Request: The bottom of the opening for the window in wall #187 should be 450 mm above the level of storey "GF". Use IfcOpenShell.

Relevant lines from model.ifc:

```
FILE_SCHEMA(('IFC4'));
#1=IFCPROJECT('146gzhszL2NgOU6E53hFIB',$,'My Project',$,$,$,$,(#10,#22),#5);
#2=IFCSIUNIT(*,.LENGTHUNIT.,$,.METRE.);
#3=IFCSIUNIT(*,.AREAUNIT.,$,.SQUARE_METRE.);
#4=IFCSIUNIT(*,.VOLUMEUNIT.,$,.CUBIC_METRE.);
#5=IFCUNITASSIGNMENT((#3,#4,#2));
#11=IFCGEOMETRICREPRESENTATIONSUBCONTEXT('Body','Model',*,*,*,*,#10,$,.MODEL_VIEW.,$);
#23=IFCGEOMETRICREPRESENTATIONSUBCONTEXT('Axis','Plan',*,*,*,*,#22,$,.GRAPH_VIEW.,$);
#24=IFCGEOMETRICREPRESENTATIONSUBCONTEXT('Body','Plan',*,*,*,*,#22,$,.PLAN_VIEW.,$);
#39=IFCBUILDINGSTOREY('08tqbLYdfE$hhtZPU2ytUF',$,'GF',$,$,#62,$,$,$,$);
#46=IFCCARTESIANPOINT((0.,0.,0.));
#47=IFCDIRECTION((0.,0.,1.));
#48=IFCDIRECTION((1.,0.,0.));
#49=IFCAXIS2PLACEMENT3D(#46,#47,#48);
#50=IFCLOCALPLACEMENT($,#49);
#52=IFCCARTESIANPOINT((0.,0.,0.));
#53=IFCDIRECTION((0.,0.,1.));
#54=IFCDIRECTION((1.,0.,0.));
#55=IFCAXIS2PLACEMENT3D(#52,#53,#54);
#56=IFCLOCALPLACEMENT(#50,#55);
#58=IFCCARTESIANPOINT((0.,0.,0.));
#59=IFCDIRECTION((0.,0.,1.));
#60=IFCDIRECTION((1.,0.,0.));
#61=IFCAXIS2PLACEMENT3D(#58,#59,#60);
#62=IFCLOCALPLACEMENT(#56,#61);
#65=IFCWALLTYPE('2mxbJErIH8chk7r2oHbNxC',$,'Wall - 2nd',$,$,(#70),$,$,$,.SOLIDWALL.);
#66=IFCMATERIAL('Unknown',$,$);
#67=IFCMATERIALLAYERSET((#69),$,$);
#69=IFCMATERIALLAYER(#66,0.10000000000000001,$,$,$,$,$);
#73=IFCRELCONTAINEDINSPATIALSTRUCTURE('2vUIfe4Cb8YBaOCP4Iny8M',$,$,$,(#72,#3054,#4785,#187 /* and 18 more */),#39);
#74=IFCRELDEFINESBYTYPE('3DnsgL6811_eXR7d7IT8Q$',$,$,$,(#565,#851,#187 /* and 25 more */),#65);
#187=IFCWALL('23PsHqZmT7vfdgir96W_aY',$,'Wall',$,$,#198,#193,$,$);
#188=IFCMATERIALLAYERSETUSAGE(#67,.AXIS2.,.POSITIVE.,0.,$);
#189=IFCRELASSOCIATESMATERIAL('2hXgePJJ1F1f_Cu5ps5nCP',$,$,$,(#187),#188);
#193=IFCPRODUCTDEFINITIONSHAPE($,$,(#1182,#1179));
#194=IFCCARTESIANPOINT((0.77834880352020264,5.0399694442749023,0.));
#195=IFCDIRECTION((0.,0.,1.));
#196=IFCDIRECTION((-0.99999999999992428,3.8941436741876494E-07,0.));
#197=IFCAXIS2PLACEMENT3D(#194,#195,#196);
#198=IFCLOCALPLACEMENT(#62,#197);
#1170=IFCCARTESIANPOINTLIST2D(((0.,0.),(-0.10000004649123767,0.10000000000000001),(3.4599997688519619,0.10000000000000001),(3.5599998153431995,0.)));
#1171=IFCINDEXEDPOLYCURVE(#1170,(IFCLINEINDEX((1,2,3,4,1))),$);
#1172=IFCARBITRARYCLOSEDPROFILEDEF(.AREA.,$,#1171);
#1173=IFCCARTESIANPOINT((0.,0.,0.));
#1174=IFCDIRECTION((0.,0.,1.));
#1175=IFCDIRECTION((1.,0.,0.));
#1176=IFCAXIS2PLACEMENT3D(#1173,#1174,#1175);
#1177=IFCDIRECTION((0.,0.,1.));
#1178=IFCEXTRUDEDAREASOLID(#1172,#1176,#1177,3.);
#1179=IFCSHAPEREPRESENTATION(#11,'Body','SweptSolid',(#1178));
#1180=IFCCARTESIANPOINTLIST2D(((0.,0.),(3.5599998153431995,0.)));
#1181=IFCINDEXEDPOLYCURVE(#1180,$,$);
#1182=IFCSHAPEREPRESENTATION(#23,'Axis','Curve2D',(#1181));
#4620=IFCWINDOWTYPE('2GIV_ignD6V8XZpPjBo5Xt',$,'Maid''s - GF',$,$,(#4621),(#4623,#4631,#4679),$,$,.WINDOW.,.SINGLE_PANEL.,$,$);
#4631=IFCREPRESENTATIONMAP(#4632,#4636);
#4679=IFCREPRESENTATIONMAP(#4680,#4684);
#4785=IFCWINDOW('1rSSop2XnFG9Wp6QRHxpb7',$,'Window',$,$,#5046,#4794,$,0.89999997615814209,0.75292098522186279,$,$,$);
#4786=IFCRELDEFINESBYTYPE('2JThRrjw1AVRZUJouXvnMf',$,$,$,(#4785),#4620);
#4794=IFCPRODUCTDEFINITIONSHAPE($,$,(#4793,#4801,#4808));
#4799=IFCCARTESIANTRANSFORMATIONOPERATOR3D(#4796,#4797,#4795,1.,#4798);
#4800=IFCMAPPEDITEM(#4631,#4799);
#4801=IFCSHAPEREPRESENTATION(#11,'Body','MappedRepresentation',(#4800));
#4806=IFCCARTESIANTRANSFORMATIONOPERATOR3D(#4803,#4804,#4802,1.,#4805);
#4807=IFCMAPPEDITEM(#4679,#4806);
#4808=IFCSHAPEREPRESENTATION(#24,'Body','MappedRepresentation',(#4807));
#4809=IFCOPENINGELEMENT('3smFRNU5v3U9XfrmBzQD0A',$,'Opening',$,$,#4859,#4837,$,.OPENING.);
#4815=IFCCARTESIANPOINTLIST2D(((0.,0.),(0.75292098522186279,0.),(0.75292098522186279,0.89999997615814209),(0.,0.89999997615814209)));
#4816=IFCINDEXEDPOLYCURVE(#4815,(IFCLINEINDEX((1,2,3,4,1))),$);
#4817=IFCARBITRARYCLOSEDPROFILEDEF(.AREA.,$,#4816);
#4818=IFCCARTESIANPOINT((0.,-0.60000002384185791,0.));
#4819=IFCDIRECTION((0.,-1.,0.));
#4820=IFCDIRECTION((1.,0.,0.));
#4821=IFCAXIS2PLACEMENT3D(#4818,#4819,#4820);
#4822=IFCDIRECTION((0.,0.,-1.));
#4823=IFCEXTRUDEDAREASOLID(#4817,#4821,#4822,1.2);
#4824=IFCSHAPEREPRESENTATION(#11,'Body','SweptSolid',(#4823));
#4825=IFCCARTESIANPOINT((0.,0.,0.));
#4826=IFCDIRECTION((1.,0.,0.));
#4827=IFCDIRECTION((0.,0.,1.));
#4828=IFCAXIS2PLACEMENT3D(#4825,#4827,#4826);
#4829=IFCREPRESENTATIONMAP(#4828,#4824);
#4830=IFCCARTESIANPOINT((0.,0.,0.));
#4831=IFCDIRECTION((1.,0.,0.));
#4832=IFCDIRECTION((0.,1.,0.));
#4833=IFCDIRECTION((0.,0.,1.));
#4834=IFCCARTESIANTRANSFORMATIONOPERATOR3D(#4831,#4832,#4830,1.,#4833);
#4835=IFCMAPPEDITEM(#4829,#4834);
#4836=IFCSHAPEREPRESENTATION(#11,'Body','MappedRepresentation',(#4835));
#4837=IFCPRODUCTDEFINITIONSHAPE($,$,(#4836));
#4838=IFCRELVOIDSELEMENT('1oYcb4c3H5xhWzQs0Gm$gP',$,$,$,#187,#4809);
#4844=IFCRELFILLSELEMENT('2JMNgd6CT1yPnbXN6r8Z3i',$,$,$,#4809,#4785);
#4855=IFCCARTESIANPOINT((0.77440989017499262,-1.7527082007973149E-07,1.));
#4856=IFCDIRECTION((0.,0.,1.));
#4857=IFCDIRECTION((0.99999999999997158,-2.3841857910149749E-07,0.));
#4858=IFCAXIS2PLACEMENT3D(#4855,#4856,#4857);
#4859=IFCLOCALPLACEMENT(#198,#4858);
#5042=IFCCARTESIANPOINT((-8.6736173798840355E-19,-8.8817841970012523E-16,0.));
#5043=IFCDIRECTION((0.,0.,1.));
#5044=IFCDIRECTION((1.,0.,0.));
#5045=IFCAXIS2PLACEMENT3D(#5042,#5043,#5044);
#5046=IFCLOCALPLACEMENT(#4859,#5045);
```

```python
import numpy as np
import ifcopenshell
import ifcopenshell.api.geometry
import ifcopenshell.geom
import ifcopenshell.util.element
import ifcopenshell.util.placement
import ifcopenshell.util.shape
import ifcopenshell.util.unit

model = ifcopenshell.open("model.ifc")
unit_scale = ifcopenshell.util.unit.calculate_unit_scale(model)

window = model.by_guid("1rSSop2XnFG9Wp6QRHxpb7")
opening = window.FillsVoids[0].RelatingOpeningElement
storey = ifcopenshell.util.element.get_container(window, ifc_class="IfcBuildingStorey")
level = ifcopenshell.util.placement.get_local_placement(storey.ObjectPlacement)[2, 3]

# The opening's origin need not be at the sill, so measure its lowest point.
shape = ifcopenshell.geom.create_shape(ifcopenshell.geom.settings(), opening)
bottom = ifcopenshell.util.shape.get_shape_bottom_elevation(shape, shape.geometry) / unit_scale
dz = level + 0.45 / unit_scale - bottom

shift = np.array([0.0, 0.0, dz])
# The window is placed relative to its opening, so it follows when the opening moves.
matrix = ifcopenshell.util.placement.get_local_placement(opening.ObjectPlacement)
matrix[:3, 3] += shift
ifcopenshell.api.geometry.edit_object_placement(
    model, product=opening, matrix=matrix, is_si=False, should_transform_children=True
)

print(f"moved by {dz * unit_scale:+.3f} m")

model.write("model_v2.ifc")
```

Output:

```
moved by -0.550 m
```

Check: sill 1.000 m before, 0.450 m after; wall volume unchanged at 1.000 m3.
